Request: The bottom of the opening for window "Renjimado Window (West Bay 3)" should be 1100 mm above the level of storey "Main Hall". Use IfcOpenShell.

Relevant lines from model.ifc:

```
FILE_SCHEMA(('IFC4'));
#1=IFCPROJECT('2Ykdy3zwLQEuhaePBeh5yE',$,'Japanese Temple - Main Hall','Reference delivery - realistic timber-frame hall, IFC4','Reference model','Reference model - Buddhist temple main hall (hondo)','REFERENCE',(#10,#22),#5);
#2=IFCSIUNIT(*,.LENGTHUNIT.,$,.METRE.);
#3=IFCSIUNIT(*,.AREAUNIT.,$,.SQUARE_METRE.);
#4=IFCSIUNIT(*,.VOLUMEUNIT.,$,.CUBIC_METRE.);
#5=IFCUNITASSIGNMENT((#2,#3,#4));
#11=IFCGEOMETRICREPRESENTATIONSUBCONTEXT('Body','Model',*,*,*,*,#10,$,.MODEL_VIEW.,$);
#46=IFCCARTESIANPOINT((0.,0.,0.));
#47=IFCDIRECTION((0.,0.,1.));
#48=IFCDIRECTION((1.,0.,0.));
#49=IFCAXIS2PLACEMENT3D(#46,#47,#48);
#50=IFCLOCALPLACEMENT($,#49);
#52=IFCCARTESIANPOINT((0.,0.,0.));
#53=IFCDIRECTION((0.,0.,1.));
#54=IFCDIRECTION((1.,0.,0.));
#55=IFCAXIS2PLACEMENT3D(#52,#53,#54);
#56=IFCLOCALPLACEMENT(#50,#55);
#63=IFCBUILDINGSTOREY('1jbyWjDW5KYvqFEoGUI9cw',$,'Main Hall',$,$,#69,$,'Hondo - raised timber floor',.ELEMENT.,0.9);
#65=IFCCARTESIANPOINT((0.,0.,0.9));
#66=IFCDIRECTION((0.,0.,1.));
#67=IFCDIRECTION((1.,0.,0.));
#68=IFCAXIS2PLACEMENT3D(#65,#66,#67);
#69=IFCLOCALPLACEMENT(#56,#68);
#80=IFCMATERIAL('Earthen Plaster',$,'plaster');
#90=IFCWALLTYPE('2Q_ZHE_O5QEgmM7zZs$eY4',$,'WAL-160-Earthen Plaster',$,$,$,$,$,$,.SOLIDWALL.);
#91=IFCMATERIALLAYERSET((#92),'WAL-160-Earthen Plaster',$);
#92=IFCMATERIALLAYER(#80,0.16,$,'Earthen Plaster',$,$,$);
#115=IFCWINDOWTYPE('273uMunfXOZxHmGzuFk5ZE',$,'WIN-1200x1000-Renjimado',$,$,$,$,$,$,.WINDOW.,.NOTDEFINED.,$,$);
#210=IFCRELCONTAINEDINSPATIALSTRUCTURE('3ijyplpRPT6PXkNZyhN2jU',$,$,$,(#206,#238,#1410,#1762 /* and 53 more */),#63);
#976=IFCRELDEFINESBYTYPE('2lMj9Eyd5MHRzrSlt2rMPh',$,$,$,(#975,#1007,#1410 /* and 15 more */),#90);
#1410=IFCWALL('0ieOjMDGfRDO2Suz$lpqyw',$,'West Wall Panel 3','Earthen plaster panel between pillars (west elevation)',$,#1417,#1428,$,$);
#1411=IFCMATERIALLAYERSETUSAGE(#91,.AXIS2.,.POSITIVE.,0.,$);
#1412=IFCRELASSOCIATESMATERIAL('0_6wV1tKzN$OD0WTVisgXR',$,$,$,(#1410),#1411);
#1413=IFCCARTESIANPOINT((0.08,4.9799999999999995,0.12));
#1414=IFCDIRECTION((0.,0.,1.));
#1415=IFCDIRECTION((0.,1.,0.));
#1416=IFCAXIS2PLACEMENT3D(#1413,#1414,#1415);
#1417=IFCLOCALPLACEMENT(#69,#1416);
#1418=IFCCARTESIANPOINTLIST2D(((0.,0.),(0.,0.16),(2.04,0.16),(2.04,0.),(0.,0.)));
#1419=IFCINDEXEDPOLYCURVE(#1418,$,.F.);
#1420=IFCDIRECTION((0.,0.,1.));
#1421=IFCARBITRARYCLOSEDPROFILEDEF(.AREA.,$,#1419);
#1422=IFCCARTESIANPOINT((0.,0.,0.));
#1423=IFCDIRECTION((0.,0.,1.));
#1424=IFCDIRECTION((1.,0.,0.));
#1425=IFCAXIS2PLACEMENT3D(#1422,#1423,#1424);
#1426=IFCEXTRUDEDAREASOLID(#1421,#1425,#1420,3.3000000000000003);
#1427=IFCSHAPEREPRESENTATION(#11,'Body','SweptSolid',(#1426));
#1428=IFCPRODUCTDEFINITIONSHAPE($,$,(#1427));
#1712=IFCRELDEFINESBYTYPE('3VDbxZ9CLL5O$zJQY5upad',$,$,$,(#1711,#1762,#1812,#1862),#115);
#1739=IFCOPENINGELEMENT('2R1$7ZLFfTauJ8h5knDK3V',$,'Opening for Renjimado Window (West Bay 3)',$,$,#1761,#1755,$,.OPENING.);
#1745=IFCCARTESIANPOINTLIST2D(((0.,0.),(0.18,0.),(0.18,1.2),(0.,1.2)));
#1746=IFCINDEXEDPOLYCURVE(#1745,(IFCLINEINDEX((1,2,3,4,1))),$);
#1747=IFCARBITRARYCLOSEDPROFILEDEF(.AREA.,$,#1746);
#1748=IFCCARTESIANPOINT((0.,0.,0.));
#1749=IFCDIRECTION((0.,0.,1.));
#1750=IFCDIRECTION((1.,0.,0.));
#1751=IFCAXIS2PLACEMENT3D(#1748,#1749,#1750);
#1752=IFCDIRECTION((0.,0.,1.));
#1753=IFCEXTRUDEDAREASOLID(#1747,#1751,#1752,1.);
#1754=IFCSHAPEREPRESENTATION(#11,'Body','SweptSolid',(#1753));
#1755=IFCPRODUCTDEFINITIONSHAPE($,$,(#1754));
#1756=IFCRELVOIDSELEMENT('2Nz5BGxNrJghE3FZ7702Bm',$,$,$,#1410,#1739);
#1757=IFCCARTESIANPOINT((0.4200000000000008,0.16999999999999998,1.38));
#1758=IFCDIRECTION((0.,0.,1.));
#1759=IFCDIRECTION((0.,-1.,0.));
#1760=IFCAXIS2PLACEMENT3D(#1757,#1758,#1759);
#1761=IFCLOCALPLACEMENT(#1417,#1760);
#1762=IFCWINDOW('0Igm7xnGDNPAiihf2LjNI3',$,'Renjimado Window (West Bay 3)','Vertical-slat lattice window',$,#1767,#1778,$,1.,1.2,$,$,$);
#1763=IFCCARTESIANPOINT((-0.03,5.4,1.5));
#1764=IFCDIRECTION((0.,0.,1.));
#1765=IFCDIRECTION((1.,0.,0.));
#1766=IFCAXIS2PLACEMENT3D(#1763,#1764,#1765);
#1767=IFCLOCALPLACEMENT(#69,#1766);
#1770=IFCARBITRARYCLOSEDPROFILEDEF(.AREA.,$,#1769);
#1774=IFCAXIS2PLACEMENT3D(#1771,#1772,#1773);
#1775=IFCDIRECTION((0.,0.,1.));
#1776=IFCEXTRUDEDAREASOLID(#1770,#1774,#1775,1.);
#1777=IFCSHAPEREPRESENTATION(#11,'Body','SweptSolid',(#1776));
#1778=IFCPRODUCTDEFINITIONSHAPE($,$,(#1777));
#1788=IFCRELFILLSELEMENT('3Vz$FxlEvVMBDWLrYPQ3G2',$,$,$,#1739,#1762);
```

```python
import numpy as np
import ifcopenshell
import ifcopenshell.api.geometry
import ifcopenshell.geom
import ifcopenshell.util.element
import ifcopenshell.util.placement
import ifcopenshell.util.shape
import ifcopenshell.util.unit

model = ifcopenshell.open("model.ifc")
unit_scale = ifcopenshell.util.unit.calculate_unit_scale(model)

window = model.by_id(1762)
opening = window.FillsVoids[0].RelatingOpeningElement
storey = ifcopenshell.util.element.get_container(window, ifc_class="IfcBuildingStorey")
level = ifcopenshell.util.placement.get_local_placement(storey.ObjectPlacement)[2, 3]

# The opening's origin need not be at the sill, so measure its lowest point.
shape = ifcopenshell.geom.create_shape(ifcopenshell.geom.settings(), opening)
bottom = ifcopenshell.util.shape.get_shape_bottom_elevation(shape, shape.geometry) / unit_scale
dz = level + 1.1 / unit_scale - bottom

shift = np.array([0.0, 0.0, dz])
# The window is not placed relative to its opening, so move both.
for product in (opening, window):
    matrix = ifcopenshell.util.placement.get_local_placement(product.ObjectPlacement)
    matrix[:3, 3] += shift
    ifcopenshell.api.geometry.edit_object_placement(model, product=product, matrix=matrix, is_si=False)

print(f"moved by {dz * unit_scale:+.3f} m")

model.write("model_v2.ifc")
```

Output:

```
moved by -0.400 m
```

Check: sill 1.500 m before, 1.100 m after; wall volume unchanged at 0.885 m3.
